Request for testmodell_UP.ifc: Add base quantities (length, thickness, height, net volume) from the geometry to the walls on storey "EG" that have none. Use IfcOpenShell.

First a look at what the model holds.

```python
import ifcopenshell
import ifcopenshell.util.element
import ifcopenshell.util.unit

model = ifcopenshell.open("testmodell_UP.ifc")
print(model.schema)
for unit_type in ("LENGTHUNIT", "AREAUNIT", "VOLUMEUNIT"):
    print(unit_type, ifcopenshell.util.unit.calculate_unit_scale(model, unit_type))
storey = next(s for s in model.by_type("IfcBuildingStorey") if s.Name == "EG")
walls = [e for e in ifcopenshell.util.element.get_decomposition(storey) if e.is_a("IfcWall")]
for e in sorted(walls, key=lambda e: e.id()):
    print(e.id(), e.is_a(), e.Name, list(ifcopenshell.util.element.get_psets(e, qtos_only=True)), sep=" | ")
```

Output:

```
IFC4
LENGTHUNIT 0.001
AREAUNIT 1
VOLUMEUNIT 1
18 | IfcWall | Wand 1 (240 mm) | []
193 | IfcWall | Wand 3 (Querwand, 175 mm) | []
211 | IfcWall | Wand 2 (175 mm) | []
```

```python
import ifcopenshell
import ifcopenshell.api.pset
import ifcopenshell.geom
import ifcopenshell.util.element
import ifcopenshell.util.shape
import ifcopenshell.util.unit

model = ifcopenshell.open("testmodell_UP.ifc")
unit_scale = ifcopenshell.util.unit.calculate_unit_scale(model)
volume_scale = ifcopenshell.util.unit.calculate_unit_scale(model, "VOLUMEUNIT")
settings = ifcopenshell.geom.settings()

storey = next(s for s in model.by_type("IfcBuildingStorey") if s.Name == "EG")
walls = [e for e in ifcopenshell.util.element.get_decomposition(storey) if e.is_a("IfcWall")]

for e in sorted(walls, key=lambda e: e.id()):
    if ifcopenshell.util.element.get_psets(e, qtos_only=True, should_inherit=False):
        continue
    # Geometry comes back in metres, in the element's own axes.
    shape = ifcopenshell.geom.create_shape(settings, e)
    values = {
        "Length": ifcopenshell.util.shape.get_x(shape.geometry) / unit_scale,
        "Width": ifcopenshell.util.shape.get_y(shape.geometry) / unit_scale,
        "Height": ifcopenshell.util.shape.get_z(shape.geometry) / unit_scale,
        "NetVolume": ifcopenshell.util.shape.get_volume(shape.geometry) / volume_scale,
    }
    qto = ifcopenshell.api.pset.add_qto(model, product=e, name="Qto_WallBaseQuantities")
    ifcopenshell.api.pset.edit_qto(model, qto=qto, properties=values)
    print(e.id(), {k: round(v, 3) for k, v in values.items()})

model.write("testmodell_UP_edited.ifc")
```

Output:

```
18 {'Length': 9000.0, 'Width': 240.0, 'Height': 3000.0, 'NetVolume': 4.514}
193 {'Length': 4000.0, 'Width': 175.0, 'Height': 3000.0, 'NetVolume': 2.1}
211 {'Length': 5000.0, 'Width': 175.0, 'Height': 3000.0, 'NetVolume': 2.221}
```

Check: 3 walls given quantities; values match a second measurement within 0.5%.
